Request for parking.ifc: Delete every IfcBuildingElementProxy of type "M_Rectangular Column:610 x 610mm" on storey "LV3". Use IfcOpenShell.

First a look at what the model holds.

```python
import ifcopenshell
import ifcopenshell.util.element

model = ifcopenshell.open("parking.ifc")
print(model.schema)
storey = next(s for s in model.by_type("IfcBuildingStorey") if s.Name == "LV3")
proxies = [e for e in ifcopenshell.util.element.get_decomposition(storey) if e.is_a("IfcBuildingElementProxy")]
seen = {}
for e in proxies:
    element_type = ifcopenshell.util.element.get_type(e)
    name = element_type.Name if element_type not in (None, e) else None
    seen[name] = seen.get(name, 0) + 1
for name, count in sorted(seen.items(), key=str):
    print(count, "x", name)
```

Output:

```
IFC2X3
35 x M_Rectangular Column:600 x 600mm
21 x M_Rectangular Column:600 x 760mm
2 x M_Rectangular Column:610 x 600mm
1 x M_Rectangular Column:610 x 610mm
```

```python
import ifcopenshell
import ifcopenshell.api.root
import ifcopenshell.util.element

model = ifcopenshell.open("parking.ifc")

storey = next(s for s in model.by_type("IfcBuildingStorey") if s.Name == "LV3")
proxies = [e for e in ifcopenshell.util.element.get_decomposition(storey) if e.is_a("IfcBuildingElementProxy")]
targets = [e for e in proxies if (t := ifcopenshell.util.element.get_type(e)) not in (None, e) and t.Name == "M_Rectangular Column:610 x 610mm"]

for e in targets:
    ifcopenshell.api.root.remove_product(model, product=e)
print(len(targets), "removed")

model.write("parking_edited.ifc")
```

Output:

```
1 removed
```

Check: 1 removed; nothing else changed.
